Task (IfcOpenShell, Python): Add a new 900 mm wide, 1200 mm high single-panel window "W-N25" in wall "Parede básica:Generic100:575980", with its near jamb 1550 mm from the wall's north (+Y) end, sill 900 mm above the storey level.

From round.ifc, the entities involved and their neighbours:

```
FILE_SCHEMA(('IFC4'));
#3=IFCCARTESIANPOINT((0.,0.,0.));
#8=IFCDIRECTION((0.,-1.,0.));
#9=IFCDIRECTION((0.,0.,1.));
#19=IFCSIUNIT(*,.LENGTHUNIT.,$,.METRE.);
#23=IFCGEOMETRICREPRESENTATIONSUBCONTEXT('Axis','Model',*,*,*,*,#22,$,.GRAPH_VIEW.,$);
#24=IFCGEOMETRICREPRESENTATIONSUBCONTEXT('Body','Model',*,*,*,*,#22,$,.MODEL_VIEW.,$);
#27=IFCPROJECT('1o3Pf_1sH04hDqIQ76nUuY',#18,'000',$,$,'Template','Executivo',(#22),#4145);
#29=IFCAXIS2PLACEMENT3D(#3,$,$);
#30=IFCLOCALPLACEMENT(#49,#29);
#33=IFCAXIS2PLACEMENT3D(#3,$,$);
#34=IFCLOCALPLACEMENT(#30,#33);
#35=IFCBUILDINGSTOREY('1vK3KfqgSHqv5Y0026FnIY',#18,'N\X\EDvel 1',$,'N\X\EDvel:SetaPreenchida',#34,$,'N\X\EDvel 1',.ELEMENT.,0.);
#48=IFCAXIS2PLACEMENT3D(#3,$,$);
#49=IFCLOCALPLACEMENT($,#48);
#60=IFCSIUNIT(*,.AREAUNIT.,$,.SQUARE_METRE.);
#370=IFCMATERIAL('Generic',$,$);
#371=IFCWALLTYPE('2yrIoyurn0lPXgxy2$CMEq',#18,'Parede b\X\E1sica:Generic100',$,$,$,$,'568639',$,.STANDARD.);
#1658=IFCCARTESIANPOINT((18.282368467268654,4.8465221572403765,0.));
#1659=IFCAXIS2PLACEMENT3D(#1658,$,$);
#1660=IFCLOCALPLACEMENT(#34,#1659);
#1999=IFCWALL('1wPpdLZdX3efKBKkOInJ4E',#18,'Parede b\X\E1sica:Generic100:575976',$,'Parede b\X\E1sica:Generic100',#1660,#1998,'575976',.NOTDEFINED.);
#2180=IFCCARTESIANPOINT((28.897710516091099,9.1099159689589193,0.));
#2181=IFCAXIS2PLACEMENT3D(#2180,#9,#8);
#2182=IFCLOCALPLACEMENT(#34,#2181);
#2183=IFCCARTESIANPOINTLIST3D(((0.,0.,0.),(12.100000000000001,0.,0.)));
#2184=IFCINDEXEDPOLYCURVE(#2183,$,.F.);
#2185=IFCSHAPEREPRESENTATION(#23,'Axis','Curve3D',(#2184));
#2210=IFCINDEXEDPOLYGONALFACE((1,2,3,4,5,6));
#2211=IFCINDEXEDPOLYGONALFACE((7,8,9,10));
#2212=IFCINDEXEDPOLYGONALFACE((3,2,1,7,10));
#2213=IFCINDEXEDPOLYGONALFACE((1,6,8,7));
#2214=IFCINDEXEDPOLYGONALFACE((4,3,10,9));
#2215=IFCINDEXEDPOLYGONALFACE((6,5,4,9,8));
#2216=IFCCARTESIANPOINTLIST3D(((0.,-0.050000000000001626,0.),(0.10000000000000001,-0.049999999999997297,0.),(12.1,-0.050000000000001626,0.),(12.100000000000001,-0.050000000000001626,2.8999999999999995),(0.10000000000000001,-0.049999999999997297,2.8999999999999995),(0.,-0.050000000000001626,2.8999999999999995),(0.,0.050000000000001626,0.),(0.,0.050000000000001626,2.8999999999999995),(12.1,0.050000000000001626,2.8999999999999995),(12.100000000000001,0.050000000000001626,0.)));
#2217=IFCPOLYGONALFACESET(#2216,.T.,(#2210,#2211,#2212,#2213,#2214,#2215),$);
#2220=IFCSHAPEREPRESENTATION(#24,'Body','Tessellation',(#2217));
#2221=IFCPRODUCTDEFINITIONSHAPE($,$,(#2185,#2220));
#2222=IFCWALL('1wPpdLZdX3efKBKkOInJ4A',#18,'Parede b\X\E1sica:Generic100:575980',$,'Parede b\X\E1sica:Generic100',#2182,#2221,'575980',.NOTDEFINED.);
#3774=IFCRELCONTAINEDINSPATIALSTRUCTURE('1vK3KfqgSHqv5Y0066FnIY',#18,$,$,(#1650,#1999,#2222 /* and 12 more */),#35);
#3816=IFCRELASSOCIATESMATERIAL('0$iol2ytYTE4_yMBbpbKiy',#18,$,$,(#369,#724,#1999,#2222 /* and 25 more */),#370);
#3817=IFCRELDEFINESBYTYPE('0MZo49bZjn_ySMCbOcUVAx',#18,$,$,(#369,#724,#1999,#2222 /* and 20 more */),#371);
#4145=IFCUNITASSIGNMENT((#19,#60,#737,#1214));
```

```python
import numpy as np
import ifcopenshell
import ifcopenshell.api.feature
import ifcopenshell.api.geometry
import ifcopenshell.api.root
import ifcopenshell.api.spatial
import ifcopenshell.geom
import ifcopenshell.util.element
import ifcopenshell.util.placement
import ifcopenshell.util.representation
import ifcopenshell.util.shape
import ifcopenshell.util.unit

model = ifcopenshell.open("round.ifc")
unit_scale = ifcopenshell.util.unit.calculate_unit_scale(model)
settings = ifcopenshell.geom.settings()


def volume(element):
    """Net volume in cubic metres, openings subtracted."""
    shape = ifcopenshell.geom.create_shape(settings, element)
    return ifcopenshell.util.shape.get_volume(shape.geometry)


wall = model.by_guid("1wPpdLZdX3efKBKkOInJ4A")
storey = ifcopenshell.util.element.get_container(wall, ifc_class="IfcBuildingStorey")
context = ifcopenshell.util.representation.get_context(model, "Model", "Body", "MODEL_VIEW")
before = volume(wall)

width, height, from_end, sill = 0.9, 1.2, 1.55, 0.9  # metres

# The wall runs along its own X axis, and the end named is its -X end.
wall_shape = ifcopenshell.geom.create_shape(settings, wall)
x, y, z = ifcopenshell.util.shape.get_vertices(wall_shape.geometry).T
start = x.min() + from_end
face, thickness = float(y.min()), float(y.max() - y.min())
wall_matrix = ifcopenshell.util.placement.get_local_placement(wall.ObjectPlacement)
level = ifcopenshell.util.placement.get_local_placement(storey.ObjectPlacement)[2, 3]


def in_wall(x, y):
    """Placement at x, y metres in the wall's axes, at sill height."""
    matrix = wall_matrix.copy()
    matrix[:, 3] = wall_matrix @ np.array([x / unit_scale, y / unit_scale, 0.0, 1.0])
    matrix[2, 3] = level + sill / unit_scale
    return matrix


# Opening: a box that overshoots both wall faces by 50 mm.
opening = ifcopenshell.api.root.create_entity(model, ifc_class="IfcOpeningElement", predefined_type="OPENING")
box = ifcopenshell.api.geometry.add_wall_representation(
    model, context=context, length=width, height=height, thickness=thickness + 0.1
)
ifcopenshell.api.geometry.assign_representation(model, product=opening, representation=box)
ifcopenshell.api.geometry.edit_object_placement(model, product=opening, matrix=in_wall(start, face - 0.05), is_si=False)
ifcopenshell.api.feature.add_feature(model, feature=opening, element=wall)

window = ifcopenshell.api.root.create_entity(model, ifc_class="IfcWindow", name="W-N25", predefined_type="WINDOW")
window.OverallWidth, window.OverallHeight = width / unit_scale, height / unit_scale
window.PartitioningType = "SINGLE_PANEL"
body = ifcopenshell.api.geometry.add_window_representation(
    model,
    context=context,
    overall_width=window.OverallWidth,
    overall_height=window.OverallHeight,
    partition_type="SINGLE_PANEL",
)
ifcopenshell.api.geometry.assign_representation(model, product=window, representation=body)
ifcopenshell.api.spatial.assign_container(model, products=[window], relating_structure=storey)
ifcopenshell.api.feature.add_filling(model, opening=opening, element=window)

# Centre the window in the wall's thickness.
ifcopenshell.api.geometry.edit_object_placement(model, product=window, matrix=in_wall(start, face), is_si=False)
window_shape = ifcopenshell.geom.create_shape(settings, window)
depth = ifcopenshell.util.shape.get_vertices(window_shape.geometry)[:, 1]
offset = face + thickness / 2 - (depth.min() + depth.max()) / 2
ifcopenshell.api.geometry.edit_object_placement(model, product=window, matrix=in_wall(start, offset), is_si=False)

after = volume(wall)

print(f"wall volume {before:.3f} -> {after:.3f} m3")

model.write("round_v2.ifc")
```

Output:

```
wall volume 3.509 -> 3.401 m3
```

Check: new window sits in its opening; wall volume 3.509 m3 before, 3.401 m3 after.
